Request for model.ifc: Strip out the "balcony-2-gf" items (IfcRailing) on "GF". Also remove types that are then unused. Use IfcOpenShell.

First a look at what the model holds.

```python
import ifcopenshell
import ifcopenshell.util.element

model = ifcopenshell.open("model.ifc")
print(model.schema)
storey = next(s for s in model.by_type("IfcBuildingStorey") if s.Name == "GF")
railings = [e for e in ifcopenshell.util.element.get_decomposition(storey) if e.is_a("IfcRailing")]
seen = {}
for e in railings:
    element_type = ifcopenshell.util.element.get_type(e)
    name = element_type.Name if element_type not in (None, e) else None
    seen[name] = seen.get(name, 0) + 1
for name, count in sorted(seen.items(), key=str):
    print(count, "x", name)
```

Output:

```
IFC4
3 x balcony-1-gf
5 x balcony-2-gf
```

```python
import ifcopenshell
import ifcopenshell.api.root
import ifcopenshell.util.element

model = ifcopenshell.open("model.ifc")

storey = next(s for s in model.by_type("IfcBuildingStorey") if s.Name == "GF")
railings = [e for e in ifcopenshell.util.element.get_decomposition(storey) if e.is_a("IfcRailing")]
targets = [e for e in railings if (t := ifcopenshell.util.element.get_type(e)) not in (None, e) and t.Name == "balcony-2-gf"]
types = {ifcopenshell.util.element.get_type(e) for e in targets} - {None, *targets}

for e in targets:
    ifcopenshell.api.root.remove_product(model, product=e)
print(len(targets), "removed")

unused = [t for t in types if not ifcopenshell.util.element.get_types(t)]
for t in unused:
    ifcopenshell.api.root.remove_product(model, product=t)
print(len(unused), "unused types removed")

model.write("model_updated.ifc")
```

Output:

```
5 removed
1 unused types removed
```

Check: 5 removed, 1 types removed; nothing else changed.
